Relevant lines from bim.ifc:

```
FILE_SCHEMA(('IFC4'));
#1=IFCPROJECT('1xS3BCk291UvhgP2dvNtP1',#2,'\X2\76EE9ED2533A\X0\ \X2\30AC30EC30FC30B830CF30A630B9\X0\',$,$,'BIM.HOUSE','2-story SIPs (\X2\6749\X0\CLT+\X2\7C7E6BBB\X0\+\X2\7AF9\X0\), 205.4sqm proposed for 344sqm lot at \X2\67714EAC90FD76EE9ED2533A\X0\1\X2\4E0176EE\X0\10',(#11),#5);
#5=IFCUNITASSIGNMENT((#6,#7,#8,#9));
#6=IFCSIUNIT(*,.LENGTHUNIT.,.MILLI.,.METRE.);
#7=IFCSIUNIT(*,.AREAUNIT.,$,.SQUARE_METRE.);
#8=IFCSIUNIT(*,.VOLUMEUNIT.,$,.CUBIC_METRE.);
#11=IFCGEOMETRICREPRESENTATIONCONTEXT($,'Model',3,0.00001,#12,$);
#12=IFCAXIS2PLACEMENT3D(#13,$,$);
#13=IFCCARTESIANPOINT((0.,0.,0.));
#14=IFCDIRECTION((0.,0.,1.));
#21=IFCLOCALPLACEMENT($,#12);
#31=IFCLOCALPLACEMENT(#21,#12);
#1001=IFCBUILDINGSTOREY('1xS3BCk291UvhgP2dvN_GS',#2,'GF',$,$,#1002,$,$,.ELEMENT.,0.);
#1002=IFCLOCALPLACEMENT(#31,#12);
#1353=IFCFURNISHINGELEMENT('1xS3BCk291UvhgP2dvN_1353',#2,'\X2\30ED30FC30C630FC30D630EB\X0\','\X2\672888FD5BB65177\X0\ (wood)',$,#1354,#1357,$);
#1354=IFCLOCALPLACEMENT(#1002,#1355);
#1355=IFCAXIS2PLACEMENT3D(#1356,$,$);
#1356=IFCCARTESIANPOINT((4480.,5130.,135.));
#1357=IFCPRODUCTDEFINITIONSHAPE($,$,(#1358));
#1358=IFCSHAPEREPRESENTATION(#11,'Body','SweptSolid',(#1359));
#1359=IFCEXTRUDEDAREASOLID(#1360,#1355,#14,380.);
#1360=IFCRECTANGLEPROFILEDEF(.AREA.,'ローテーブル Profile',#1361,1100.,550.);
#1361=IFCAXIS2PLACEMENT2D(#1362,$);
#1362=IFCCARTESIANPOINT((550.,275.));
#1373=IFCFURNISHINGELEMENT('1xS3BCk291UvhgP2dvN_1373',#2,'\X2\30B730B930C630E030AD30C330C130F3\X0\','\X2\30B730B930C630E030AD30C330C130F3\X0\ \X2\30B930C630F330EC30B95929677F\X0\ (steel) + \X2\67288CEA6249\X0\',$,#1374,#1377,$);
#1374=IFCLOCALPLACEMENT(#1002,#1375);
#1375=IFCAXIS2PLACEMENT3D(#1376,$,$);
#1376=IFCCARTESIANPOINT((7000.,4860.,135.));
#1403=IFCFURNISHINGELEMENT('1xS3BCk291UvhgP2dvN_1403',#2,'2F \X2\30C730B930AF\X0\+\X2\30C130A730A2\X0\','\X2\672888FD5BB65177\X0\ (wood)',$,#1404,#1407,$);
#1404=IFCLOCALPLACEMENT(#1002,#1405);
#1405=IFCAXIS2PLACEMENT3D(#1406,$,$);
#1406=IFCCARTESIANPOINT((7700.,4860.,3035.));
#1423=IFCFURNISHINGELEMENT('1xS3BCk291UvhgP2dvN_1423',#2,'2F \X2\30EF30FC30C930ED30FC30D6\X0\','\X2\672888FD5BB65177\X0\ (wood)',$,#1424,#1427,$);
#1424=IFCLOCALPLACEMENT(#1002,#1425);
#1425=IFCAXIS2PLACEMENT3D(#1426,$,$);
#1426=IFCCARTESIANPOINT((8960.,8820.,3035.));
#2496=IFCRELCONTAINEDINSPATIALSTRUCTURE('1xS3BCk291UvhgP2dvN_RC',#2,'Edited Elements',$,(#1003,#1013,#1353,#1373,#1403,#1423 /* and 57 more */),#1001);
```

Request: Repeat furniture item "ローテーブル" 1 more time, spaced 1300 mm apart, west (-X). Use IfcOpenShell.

```python
import numpy as np
import ifcopenshell
import ifcopenshell.api.geometry
import ifcopenshell.api.root
import ifcopenshell.util.element
import ifcopenshell.util.placement

model = ifcopenshell.open("bim.ifc")


def reuse_history(source, copy):
    """copy_class also copies each property set's owner history, people and application; keep the originals."""
    for rel in copy.IsDefinedBy:
        if rel.is_a("IfcRelDefinesByProperties") and (history := rel.RelatingPropertyDefinition.OwnerHistory):
            rel.RelatingPropertyDefinition.OwnerHistory = source.OwnerHistory
            ifcopenshell.util.element.remove_deep2(model, history)


source = model.by_guid("1xS3BCk291UvhgP2dvN_1353")
base = ifcopenshell.util.placement.get_local_placement(source.ObjectPlacement)
step = np.array([-1.0, 0.0, 0.0]) * 1300.0

for i in range(1, 2):
    copy = ifcopenshell.api.root.copy_class(model, product=source)
    copy.Representation = ifcopenshell.util.element.copy_deep(
        model, source.Representation, exclude=["IfcGeometricRepresentationContext", "IfcRepresentationMap"]
    )
    reuse_history(source, copy)
    matrix = base.copy()
    matrix[:3, 3] += i * step
    print("added at", matrix[:3, 3].round(3) + 0.0)
    ifcopenshell.api.geometry.edit_object_placement(model, product=copy, matrix=matrix, is_si=False)

model.write("bim_v2.ifc")
```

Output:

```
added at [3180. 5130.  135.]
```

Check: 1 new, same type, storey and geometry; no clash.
